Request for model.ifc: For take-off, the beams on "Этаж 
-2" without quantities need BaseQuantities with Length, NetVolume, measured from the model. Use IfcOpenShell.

First a look at what the model holds.

```python
import ifcopenshell
import ifcopenshell.util.element
import ifcopenshell.util.unit

model = ifcopenshell.open("model.ifc")
print(model.schema)
for unit_type in ("LENGTHUNIT", "AREAUNIT", "VOLUMEUNIT"):
    print(unit_type, ifcopenshell.util.unit.calculate_unit_scale(model, unit_type))
storey = next(s for s in model.by_type("IfcBuildingStorey") if s.Name == 'Этаж \r\n-2')
beams = [e for e in ifcopenshell.util.element.get_decomposition(storey) if e.is_a("IfcBeam")]
for e in sorted(beams, key=lambda e: e.id()):
    print(e.id(), e.is_a(), e.Name, list(ifcopenshell.util.element.get_psets(e, qtos_only=True)), sep=" | ")
```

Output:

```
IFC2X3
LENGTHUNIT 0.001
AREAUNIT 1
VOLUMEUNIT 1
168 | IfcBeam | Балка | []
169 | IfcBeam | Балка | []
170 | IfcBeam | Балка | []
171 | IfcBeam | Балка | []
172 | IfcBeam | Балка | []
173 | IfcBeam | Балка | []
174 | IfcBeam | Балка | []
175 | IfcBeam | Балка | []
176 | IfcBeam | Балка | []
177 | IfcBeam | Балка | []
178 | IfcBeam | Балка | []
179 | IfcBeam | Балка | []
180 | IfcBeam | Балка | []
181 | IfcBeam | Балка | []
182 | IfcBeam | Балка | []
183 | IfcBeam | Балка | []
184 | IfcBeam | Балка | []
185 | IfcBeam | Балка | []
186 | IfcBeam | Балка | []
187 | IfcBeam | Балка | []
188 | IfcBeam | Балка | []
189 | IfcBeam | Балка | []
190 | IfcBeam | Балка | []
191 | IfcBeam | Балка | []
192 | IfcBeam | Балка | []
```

```python
import ifcopenshell
import ifcopenshell.api.pset
import ifcopenshell.geom
import ifcopenshell.util.element
import ifcopenshell.util.shape
import ifcopenshell.util.unit

model = ifcopenshell.open("model.ifc")
unit_scale = ifcopenshell.util.unit.calculate_unit_scale(model)
volume_scale = ifcopenshell.util.unit.calculate_unit_scale(model, "VOLUMEUNIT")
settings = ifcopenshell.geom.settings()

storey = next(s for s in model.by_type("IfcBuildingStorey") if s.Name == 'Этаж \r\n-2')
beams = [e for e in ifcopenshell.util.element.get_decomposition(storey) if e.is_a("IfcBeam")]

for e in sorted(beams, key=lambda e: e.id()):
    if ifcopenshell.util.element.get_psets(e, qtos_only=True, should_inherit=False):
        continue
    # Geometry comes back in metres, in the element's own axes.
    shape = ifcopenshell.geom.create_shape(settings, e)
    values = {
        "Length": ifcopenshell.util.shape.get_max_xyz(shape.geometry) / unit_scale,
        "NetVolume": ifcopenshell.util.shape.get_volume(shape.geometry) / volume_scale,
    }
    qto = ifcopenshell.api.pset.add_qto(model, product=e, name="BaseQuantities")
    ifcopenshell.api.pset.edit_qto(model, qto=qto, properties=values)
    print(e.id(), {k: round(v, 3) for k, v in values.items()})

model.write("model-out.ifc")
```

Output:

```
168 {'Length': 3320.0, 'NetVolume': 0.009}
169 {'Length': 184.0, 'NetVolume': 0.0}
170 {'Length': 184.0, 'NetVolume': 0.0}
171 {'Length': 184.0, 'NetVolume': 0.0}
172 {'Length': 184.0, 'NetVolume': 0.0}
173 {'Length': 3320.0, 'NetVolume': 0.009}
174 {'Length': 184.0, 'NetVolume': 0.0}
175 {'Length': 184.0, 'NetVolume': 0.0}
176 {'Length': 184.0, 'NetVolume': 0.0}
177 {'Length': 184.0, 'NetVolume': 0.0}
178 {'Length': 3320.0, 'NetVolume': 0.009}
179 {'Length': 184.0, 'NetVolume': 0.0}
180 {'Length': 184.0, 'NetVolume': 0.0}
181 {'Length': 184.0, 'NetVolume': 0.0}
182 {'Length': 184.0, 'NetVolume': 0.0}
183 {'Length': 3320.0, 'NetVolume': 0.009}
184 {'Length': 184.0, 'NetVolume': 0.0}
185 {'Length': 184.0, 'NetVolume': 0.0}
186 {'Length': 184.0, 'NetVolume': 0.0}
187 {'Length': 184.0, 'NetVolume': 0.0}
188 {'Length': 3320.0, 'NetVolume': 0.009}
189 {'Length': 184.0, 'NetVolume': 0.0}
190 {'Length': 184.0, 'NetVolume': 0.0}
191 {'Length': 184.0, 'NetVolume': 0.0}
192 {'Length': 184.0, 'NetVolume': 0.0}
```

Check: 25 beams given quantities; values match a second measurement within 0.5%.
